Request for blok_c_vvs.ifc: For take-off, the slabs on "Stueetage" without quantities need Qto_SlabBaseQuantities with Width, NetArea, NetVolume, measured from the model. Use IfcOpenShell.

First a look at what the model holds.

```python
import ifcopenshell
import ifcopenshell.util.element
import ifcopenshell.util.unit

model = ifcopenshell.open("blok_c_vvs.ifc")
print(model.schema)
for unit_type in ("LENGTHUNIT", "AREAUNIT", "VOLUMEUNIT"):
    print(unit_type, ifcopenshell.util.unit.calculate_unit_scale(model, unit_type))
storey = next(s for s in model.by_type("IfcBuildingStorey") if s.Name == "Stueetage")
slabs = [e for e in ifcopenshell.util.element.get_decomposition(storey) if e.is_a("IfcSlab")]
for e in sorted(slabs, key=lambda e: e.id()):
    print(e.id(), e.is_a(), e.Name, list(ifcopenshell.util.element.get_psets(e, qtos_only=True)), sep=" | ")
```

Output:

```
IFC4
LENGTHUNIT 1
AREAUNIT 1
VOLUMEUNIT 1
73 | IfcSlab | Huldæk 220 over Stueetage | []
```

```python
import ifcopenshell
import ifcopenshell.api.pset
import ifcopenshell.geom
import ifcopenshell.util.element
import ifcopenshell.util.shape
import ifcopenshell.util.unit

model = ifcopenshell.open("blok_c_vvs.ifc")
unit_scale = ifcopenshell.util.unit.calculate_unit_scale(model)
area_scale = ifcopenshell.util.unit.calculate_unit_scale(model, "AREAUNIT")
volume_scale = ifcopenshell.util.unit.calculate_unit_scale(model, "VOLUMEUNIT")
settings = ifcopenshell.geom.settings()

storey = next(s for s in model.by_type("IfcBuildingStorey") if s.Name == "Stueetage")
slabs = [e for e in ifcopenshell.util.element.get_decomposition(storey) if e.is_a("IfcSlab")]

for e in sorted(slabs, key=lambda e: e.id()):
    if ifcopenshell.util.element.get_psets(e, qtos_only=True, should_inherit=False):
        continue
    # Geometry comes back in metres, in the element's own axes.
    shape = ifcopenshell.geom.create_shape(settings, e)
    values = {
        "Width": ifcopenshell.util.shape.get_z(shape.geometry) / unit_scale,
        "NetArea": ifcopenshell.util.shape.get_footprint_area(shape.geometry) / area_scale,
        "NetVolume": ifcopenshell.util.shape.get_volume(shape.geometry) / volume_scale,
    }
    qto = ifcopenshell.api.pset.add_qto(model, product=e, name="Qto_SlabBaseQuantities")
    ifcopenshell.api.pset.edit_qto(model, qto=qto, properties=values)
    print(e.id(), {k: round(v, 3) for k, v in values.items()})

model.write("blok_c_vvs_v2.ifc")
```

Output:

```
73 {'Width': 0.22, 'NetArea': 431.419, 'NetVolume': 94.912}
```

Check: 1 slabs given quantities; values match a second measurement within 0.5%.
